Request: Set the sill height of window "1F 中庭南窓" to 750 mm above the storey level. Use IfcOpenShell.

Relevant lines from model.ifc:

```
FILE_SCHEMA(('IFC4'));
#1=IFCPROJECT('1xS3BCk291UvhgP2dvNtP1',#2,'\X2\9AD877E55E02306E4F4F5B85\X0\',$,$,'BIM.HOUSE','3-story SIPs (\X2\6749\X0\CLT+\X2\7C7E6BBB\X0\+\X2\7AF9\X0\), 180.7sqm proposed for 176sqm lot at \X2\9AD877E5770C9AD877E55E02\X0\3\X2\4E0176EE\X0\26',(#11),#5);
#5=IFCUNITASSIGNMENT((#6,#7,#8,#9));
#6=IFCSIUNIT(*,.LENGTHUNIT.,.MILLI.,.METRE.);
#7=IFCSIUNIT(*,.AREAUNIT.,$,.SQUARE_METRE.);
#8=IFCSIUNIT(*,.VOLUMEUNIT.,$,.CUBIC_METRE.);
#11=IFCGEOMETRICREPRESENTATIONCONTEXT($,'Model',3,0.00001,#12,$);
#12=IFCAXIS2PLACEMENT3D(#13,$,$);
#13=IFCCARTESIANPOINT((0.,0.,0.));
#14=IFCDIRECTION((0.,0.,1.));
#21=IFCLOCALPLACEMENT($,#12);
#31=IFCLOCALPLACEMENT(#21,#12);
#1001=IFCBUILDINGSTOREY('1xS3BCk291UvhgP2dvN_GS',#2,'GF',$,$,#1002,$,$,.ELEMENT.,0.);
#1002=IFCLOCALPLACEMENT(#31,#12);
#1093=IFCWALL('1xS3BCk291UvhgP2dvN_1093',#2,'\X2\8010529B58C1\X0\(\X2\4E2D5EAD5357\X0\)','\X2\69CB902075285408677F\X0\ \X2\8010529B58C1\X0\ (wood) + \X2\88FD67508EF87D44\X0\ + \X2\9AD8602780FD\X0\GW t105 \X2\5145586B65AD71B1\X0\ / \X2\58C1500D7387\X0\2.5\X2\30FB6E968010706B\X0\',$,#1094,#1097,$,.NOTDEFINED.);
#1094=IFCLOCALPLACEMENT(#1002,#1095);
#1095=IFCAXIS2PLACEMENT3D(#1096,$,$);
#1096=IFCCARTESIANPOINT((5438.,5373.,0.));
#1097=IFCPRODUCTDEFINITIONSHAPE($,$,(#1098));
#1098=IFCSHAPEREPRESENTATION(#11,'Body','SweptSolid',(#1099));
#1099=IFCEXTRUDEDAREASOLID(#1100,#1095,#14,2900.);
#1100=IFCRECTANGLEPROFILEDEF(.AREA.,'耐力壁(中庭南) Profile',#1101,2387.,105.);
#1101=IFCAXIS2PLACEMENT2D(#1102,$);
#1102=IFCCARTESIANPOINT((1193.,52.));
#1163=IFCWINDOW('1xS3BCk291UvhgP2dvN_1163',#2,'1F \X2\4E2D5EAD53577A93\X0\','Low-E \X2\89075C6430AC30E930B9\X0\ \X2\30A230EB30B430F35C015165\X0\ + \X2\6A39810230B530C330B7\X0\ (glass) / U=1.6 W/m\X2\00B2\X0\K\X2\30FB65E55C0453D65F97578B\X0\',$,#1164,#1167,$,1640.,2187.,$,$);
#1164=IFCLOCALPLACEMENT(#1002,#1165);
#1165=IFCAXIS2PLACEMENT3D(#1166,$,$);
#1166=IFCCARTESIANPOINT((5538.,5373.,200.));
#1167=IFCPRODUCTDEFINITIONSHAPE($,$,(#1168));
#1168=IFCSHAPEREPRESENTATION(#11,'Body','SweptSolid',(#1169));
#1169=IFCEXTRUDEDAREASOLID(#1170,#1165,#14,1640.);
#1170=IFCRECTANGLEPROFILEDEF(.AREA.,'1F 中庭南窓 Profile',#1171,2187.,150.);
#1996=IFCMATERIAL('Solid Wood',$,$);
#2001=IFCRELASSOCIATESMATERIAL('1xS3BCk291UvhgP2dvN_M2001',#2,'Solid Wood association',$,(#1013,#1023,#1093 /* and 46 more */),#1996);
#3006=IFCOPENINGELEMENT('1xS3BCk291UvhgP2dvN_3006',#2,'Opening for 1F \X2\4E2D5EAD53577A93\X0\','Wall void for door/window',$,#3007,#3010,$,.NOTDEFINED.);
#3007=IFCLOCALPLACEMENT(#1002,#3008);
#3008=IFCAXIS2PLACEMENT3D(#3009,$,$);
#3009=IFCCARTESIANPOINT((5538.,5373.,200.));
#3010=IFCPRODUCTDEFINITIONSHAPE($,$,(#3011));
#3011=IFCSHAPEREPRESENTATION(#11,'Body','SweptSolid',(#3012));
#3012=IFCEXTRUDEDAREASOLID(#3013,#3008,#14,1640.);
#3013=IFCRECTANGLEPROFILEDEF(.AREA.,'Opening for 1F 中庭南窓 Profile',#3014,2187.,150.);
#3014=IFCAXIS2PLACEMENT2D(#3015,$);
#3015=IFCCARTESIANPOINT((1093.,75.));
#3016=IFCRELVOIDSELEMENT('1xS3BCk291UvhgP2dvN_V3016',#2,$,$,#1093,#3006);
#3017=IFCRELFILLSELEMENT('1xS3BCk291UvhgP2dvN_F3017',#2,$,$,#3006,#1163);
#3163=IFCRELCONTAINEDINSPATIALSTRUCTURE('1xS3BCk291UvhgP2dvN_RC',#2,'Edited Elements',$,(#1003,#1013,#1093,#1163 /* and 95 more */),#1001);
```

```python
import numpy as np
import ifcopenshell
import ifcopenshell.api.geometry
import ifcopenshell.geom
import ifcopenshell.util.element
import ifcopenshell.util.placement
import ifcopenshell.util.shape
import ifcopenshell.util.unit

model = ifcopenshell.open("model.ifc")
unit_scale = ifcopenshell.util.unit.calculate_unit_scale(model)

window = model.by_id(1163)
opening = window.FillsVoids[0].RelatingOpeningElement
storey = ifcopenshell.util.element.get_container(window, ifc_class="IfcBuildingStorey")
level = ifcopenshell.util.placement.get_local_placement(storey.ObjectPlacement)[2, 3]

# The opening's origin need not be at the sill, so measure its lowest point.
shape = ifcopenshell.geom.create_shape(ifcopenshell.geom.settings(), opening)
bottom = ifcopenshell.util.shape.get_shape_bottom_elevation(shape, shape.geometry) / unit_scale
dz = level + 0.75 / unit_scale - bottom

shift = np.array([0.0, 0.0, dz])
# The window is not placed relative to its opening, so move both.
for product in (opening, window):
    matrix = ifcopenshell.util.placement.get_local_placement(product.ObjectPlacement)
    matrix[:3, 3] += shift
    ifcopenshell.api.geometry.edit_object_placement(model, product=product, matrix=matrix, is_si=False)

print(f"moved by {dz * unit_scale:+.3f} m")

model.write("model_updated.ifc")
```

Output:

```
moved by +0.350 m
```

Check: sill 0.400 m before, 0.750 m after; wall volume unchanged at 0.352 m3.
